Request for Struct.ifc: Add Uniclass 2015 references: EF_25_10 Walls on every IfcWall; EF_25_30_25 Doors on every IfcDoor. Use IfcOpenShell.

First a look at what the model holds.

```python
import ifcopenshell

model = ifcopenshell.open("Struct.ifc")
print(model.schema)
print("classifications:", [c.Name for c in model.by_type("IfcClassification")])
for ifc_class in ("IfcDoor", "IfcRoof", "IfcStair", "IfcWall", "IfcWindow"):
    print(ifc_class, len(model.by_type(ifc_class)))
```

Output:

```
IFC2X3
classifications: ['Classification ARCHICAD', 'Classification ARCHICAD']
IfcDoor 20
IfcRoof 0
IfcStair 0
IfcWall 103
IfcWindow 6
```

```python
import ifcopenshell
import ifcopenshell.api.classification

model = ifcopenshell.open("Struct.ifc")

# IFC2X3 requires Source and Edition and has no link from the project to the system.
system = model.create_entity("IfcClassification", Source="NBS", Edition="2015", Name="Uniclass 2015")

codes = {
    "IfcWall": ("EF_25_10", "Walls"),
    "IfcDoor": ("EF_25_30_25", "Doors"),
}
for ifc_class, (code, name) in codes.items():
    products = model.by_type(ifc_class)
    ifcopenshell.api.classification.add_reference(
        model, products=products, classification=system, identification=code, name=name
    )
    print(code, len(products))

model.write("Struct_v2.ifc")
```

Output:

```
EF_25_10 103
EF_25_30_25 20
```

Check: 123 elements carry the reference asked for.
